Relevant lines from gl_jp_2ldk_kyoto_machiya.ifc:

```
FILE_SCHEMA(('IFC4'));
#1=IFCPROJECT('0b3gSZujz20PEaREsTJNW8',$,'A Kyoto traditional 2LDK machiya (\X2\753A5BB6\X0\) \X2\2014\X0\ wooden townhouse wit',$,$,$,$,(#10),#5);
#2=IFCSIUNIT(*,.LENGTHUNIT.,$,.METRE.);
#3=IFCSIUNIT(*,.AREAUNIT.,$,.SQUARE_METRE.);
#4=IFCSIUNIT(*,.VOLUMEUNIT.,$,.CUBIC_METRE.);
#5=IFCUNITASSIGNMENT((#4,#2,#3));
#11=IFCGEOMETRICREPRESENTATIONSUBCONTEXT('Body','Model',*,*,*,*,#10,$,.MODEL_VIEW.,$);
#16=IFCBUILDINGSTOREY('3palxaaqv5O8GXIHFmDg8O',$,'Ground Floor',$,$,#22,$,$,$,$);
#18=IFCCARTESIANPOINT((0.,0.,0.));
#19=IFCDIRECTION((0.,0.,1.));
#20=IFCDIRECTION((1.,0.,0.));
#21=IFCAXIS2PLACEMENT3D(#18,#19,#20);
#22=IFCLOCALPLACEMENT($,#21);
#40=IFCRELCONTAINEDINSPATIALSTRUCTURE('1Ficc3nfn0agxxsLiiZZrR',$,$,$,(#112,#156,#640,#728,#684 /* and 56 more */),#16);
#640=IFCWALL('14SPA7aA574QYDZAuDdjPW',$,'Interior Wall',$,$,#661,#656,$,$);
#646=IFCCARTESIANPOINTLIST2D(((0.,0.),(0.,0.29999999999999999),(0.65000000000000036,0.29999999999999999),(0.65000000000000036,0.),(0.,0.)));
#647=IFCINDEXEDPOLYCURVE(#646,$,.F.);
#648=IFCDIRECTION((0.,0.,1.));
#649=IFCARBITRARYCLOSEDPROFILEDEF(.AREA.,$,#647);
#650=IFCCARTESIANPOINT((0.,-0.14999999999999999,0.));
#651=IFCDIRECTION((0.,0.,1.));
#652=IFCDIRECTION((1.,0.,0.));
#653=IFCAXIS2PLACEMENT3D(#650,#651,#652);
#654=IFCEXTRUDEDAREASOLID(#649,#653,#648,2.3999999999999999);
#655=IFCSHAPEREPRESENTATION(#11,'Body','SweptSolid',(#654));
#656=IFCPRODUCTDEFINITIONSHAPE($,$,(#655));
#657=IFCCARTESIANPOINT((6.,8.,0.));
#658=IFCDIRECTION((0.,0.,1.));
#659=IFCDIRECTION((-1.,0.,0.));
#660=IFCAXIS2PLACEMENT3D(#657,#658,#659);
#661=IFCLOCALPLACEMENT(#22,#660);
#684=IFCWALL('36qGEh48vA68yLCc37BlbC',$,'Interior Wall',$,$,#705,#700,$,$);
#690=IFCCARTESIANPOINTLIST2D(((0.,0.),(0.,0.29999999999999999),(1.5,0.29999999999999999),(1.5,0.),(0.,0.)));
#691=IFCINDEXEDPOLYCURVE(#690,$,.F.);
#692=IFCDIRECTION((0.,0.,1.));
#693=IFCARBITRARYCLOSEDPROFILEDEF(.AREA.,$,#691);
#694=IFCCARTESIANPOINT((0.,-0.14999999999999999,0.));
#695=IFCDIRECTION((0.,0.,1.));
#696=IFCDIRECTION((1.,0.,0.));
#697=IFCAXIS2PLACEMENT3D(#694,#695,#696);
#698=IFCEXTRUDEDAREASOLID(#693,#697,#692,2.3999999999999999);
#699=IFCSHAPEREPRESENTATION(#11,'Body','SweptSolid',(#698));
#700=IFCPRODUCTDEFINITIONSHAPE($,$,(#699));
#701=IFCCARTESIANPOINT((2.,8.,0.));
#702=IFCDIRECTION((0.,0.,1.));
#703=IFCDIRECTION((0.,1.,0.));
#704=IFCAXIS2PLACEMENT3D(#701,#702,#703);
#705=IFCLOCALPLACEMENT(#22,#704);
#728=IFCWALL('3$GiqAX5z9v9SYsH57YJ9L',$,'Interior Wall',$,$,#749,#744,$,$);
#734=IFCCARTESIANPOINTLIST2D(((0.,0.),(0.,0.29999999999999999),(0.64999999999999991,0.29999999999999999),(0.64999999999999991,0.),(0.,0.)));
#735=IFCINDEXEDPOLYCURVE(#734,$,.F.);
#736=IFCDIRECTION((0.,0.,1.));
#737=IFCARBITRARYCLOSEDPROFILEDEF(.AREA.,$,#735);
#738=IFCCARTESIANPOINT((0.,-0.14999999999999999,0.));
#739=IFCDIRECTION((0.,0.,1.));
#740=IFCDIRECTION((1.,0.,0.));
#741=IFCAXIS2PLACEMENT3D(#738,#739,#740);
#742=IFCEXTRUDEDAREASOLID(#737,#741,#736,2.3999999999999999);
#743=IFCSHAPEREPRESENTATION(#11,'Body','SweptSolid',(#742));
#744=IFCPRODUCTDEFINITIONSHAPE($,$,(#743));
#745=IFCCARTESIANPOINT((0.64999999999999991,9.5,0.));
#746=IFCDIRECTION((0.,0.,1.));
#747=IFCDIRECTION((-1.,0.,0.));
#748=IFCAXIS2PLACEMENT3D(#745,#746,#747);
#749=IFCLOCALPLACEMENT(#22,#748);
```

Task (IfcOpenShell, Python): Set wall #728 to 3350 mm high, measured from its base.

```python
import ifcopenshell
import ifcopenshell.geom
import ifcopenshell.util.representation
import ifcopenshell.util.shape
import ifcopenshell.util.unit

model = ifcopenshell.open("gl_jp_2ldk_kyoto_machiya.ifc")
unit_scale = ifcopenshell.util.unit.calculate_unit_scale(model)
settings = ifcopenshell.geom.settings()


def volume(element):
    """Net volume in cubic metres, openings subtracted."""
    shape = ifcopenshell.geom.create_shape(settings, element)
    return ifcopenshell.util.shape.get_volume(shape.geometry)


wall = model.by_id(728)
before = volume(wall)

body = ifcopenshell.util.representation.get_representation(wall, "Model", "Body")
solid = body.Items[0]
old_height = solid.Depth
solid.Depth = 3.35 / unit_scale
after = volume(wall)

print(f"height {old_height:g} -> {solid.Depth:g}, volume {before:.3f} -> {after:.3f} m3")

model.write("gl_jp_2ldk_kyoto_machiya-out.ifc")
```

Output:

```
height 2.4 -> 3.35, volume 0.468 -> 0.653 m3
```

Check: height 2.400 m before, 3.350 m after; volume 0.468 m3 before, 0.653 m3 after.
